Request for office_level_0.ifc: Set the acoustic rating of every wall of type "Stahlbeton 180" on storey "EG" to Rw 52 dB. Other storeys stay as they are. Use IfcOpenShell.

First a look at what the model holds.

```python
import ifcopenshell
import ifcopenshell.util.element

model = ifcopenshell.open("office_level_0.ifc")
print(model.schema)
storey = next(s for s in model.by_type("IfcBuildingStorey") if s.Name == "EG")
walls = [e for e in ifcopenshell.util.element.get_decomposition(storey) if e.is_a("IfcWall")]
seen = {}
for e in walls:
    element_type = ifcopenshell.util.element.get_type(e)
    key = (element_type.Name if element_type != e and element_type else None, ifcopenshell.util.element.get_pset(e, "Pset_WallCommon", "AcousticRating"))
    seen[key] = seen.get(key, 0) + 1
for (name, value), count in sorted(seen.items(), key=str):
    print(count, "x", name, "|", value)
```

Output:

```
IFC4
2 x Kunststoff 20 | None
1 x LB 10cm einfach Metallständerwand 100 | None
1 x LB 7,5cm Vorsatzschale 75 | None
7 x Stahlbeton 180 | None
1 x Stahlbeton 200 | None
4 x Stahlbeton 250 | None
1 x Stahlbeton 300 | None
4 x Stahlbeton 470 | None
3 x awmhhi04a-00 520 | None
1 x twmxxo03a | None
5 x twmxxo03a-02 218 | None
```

```python
import ifcopenshell
import ifcopenshell.api.pset
import ifcopenshell.util.element

model = ifcopenshell.open("office_level_0.ifc")

storey = next(s for s in model.by_type("IfcBuildingStorey") if s.Name == "EG")
walls = [e for e in ifcopenshell.util.element.get_decomposition(storey) if e.is_a("IfcWall")]

count = 0
for e in walls:
    element_type = ifcopenshell.util.element.get_type(e)
    if element_type in (None, e) or element_type.Name != "Stahlbeton 180":
        continue
    # add_pset returns the element's existing set when there is one.
    pset = ifcopenshell.api.pset.add_pset(model, product=e, name="Pset_WallCommon")
    ifcopenshell.api.pset.edit_pset(model, pset=pset, properties={"AcousticRating": "Rw 52 dB"})
    count += 1

print(count, "walls updated")

model.write("office_level_0_v2.ifc")
```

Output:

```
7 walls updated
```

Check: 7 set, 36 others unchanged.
